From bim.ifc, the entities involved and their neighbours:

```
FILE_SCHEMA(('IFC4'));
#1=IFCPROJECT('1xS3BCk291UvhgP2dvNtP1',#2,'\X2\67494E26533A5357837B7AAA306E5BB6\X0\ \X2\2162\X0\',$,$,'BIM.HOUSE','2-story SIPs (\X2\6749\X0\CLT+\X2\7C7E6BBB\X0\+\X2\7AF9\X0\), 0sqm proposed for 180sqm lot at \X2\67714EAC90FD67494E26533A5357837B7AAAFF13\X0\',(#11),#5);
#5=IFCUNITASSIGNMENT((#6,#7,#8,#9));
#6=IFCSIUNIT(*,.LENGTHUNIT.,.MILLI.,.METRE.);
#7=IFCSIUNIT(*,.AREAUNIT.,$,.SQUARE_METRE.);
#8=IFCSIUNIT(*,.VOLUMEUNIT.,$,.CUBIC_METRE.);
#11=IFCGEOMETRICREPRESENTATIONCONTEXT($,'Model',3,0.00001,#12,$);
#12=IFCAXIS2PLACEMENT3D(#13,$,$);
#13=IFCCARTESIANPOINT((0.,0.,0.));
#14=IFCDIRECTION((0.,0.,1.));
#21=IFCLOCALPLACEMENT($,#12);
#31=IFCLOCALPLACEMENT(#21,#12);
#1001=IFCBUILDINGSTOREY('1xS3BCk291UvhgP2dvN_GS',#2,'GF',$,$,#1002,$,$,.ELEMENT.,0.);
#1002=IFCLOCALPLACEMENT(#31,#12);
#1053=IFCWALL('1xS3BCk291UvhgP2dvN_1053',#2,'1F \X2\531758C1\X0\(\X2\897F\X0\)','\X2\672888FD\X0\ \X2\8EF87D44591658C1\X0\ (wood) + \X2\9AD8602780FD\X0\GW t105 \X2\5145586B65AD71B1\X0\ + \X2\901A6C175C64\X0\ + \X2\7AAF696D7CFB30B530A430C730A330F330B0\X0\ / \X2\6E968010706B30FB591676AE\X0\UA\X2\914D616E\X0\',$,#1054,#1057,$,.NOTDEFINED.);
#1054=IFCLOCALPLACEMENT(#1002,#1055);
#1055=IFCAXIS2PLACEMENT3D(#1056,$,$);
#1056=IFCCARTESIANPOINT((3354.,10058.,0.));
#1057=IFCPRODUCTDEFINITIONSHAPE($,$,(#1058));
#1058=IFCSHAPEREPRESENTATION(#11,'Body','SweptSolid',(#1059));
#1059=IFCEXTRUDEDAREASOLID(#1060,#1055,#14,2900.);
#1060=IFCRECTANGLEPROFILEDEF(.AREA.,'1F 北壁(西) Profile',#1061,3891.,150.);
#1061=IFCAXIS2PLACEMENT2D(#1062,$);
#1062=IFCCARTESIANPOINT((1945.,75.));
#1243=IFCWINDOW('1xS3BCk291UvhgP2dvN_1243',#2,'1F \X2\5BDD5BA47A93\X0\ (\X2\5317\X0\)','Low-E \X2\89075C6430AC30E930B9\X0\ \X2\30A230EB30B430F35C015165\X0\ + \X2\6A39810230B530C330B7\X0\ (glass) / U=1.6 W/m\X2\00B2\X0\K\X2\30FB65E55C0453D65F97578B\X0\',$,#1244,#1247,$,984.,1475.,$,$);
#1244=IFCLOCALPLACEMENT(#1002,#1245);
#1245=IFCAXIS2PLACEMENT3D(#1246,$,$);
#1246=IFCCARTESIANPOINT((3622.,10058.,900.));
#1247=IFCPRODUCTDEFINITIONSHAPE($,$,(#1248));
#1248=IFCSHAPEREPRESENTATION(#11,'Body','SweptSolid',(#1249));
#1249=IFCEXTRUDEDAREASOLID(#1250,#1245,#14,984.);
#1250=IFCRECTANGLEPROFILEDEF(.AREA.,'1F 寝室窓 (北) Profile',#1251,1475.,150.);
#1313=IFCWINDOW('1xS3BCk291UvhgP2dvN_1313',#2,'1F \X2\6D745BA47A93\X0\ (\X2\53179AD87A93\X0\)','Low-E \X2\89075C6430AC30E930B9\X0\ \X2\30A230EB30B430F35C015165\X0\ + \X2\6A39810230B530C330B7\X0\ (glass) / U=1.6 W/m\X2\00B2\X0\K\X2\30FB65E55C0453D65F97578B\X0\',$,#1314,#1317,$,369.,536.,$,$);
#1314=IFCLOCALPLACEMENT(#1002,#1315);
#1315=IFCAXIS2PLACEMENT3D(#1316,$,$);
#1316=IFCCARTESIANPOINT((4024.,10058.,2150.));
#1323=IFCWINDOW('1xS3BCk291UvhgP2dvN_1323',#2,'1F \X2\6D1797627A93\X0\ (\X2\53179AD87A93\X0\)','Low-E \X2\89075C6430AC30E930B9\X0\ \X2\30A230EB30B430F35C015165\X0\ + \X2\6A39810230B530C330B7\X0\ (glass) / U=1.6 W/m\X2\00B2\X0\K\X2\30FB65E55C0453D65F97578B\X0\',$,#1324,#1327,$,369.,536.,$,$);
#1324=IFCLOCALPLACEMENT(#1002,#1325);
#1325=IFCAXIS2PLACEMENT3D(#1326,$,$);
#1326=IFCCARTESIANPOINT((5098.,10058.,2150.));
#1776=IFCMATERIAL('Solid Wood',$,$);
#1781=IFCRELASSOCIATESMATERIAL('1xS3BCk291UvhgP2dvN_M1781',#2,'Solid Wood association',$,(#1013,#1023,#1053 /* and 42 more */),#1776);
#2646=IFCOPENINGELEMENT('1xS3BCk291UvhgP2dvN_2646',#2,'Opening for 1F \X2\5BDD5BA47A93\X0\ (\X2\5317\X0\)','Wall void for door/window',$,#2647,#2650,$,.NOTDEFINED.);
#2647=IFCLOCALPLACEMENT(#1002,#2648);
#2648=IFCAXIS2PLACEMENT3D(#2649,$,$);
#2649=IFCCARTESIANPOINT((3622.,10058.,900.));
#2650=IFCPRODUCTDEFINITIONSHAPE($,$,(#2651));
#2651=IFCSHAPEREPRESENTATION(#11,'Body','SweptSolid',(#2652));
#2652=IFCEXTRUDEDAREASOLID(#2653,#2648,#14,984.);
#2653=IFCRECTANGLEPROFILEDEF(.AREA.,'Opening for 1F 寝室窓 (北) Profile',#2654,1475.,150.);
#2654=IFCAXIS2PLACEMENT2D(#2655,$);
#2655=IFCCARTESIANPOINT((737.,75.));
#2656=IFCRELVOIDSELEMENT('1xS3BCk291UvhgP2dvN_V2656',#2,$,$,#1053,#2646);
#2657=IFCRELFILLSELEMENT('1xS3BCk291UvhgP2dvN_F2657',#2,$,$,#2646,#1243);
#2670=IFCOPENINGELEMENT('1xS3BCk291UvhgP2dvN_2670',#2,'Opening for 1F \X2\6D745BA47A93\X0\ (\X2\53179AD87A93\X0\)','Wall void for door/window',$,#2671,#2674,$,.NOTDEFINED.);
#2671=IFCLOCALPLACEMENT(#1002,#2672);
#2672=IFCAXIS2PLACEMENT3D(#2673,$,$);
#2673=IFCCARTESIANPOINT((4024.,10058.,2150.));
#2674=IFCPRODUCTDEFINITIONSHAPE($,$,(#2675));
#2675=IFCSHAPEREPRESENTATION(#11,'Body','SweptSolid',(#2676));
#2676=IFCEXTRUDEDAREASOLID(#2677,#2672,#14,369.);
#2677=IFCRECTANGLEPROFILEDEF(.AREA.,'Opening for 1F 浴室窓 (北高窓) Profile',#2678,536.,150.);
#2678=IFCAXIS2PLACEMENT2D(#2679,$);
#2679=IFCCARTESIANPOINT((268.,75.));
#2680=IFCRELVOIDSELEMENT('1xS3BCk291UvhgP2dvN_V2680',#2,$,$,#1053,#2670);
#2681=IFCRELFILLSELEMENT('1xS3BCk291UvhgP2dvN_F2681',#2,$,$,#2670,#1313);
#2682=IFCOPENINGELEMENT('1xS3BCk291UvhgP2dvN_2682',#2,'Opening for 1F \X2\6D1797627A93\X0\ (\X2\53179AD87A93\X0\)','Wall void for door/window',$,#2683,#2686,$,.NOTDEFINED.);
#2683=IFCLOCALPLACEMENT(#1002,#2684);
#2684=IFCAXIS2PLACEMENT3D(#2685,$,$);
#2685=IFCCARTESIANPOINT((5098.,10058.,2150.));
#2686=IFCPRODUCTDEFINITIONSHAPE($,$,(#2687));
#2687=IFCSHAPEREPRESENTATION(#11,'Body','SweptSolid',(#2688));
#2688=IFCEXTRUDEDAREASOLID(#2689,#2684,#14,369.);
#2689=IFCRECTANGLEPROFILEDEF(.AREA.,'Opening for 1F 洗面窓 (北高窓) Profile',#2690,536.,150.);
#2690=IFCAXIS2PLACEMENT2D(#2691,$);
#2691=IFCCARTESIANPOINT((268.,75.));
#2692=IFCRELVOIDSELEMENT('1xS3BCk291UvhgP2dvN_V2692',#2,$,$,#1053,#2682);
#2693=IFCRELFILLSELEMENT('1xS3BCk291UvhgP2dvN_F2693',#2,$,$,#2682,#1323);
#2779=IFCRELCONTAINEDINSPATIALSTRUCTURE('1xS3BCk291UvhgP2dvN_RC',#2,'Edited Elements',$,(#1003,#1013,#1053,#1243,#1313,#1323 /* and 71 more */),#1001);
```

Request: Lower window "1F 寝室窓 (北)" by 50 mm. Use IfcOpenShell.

```python
import numpy as np
import ifcopenshell
import ifcopenshell.api.geometry
import ifcopenshell.util.placement
import ifcopenshell.util.unit

model = ifcopenshell.open("bim.ifc")
unit_scale = ifcopenshell.util.unit.calculate_unit_scale(model)

window = model.by_guid("1xS3BCk291UvhgP2dvN_1243")
opening = window.FillsVoids[0].RelatingOpeningElement
dz = -50.0

shift = np.array([0.0, 0.0, dz])
# The window is not placed relative to its opening, so move both.
for product in (opening, window):
    matrix = ifcopenshell.util.placement.get_local_placement(product.ObjectPlacement)
    matrix[:3, 3] += shift
    ifcopenshell.api.geometry.edit_object_placement(model, product=product, matrix=matrix, is_si=False)

print(f"moved by {dz * unit_scale:+.3f} m")

model.write("bim_updated.ifc")
```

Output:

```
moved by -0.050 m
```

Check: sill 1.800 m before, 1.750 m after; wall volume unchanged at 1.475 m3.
